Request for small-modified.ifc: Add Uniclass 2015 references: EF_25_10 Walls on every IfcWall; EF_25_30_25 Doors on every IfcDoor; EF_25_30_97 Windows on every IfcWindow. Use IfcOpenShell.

First a look at what the model holds.

```python
import ifcopenshell

model = ifcopenshell.open("small-modified.ifc")
print(model.schema)
print("classifications:", [c.Name for c in model.by_type("IfcClassification")])
for ifc_class in ("IfcDoor", "IfcRoof", "IfcStair", "IfcWall", "IfcWindow"):
    print(ifc_class, len(model.by_type(ifc_class)))
```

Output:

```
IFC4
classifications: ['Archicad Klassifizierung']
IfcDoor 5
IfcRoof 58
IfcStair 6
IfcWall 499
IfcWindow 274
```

```python
import ifcopenshell
import ifcopenshell.api.classification

model = ifcopenshell.open("small-modified.ifc")

system = ifcopenshell.api.classification.add_classification(model, classification="Uniclass 2015")

codes = {
    "IfcWall": ("EF_25_10", "Walls"),
    "IfcDoor": ("EF_25_30_25", "Doors"),
    "IfcWindow": ("EF_25_30_97", "Windows"),
}
for ifc_class, (code, name) in codes.items():
    products = model.by_type(ifc_class)
    ifcopenshell.api.classification.add_reference(
        model, products=products, classification=system, identification=code, name=name
    )
    print(code, len(products))

model.write("small-modified_rev.ifc")
```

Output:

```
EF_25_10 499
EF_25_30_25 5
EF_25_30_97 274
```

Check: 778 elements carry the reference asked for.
